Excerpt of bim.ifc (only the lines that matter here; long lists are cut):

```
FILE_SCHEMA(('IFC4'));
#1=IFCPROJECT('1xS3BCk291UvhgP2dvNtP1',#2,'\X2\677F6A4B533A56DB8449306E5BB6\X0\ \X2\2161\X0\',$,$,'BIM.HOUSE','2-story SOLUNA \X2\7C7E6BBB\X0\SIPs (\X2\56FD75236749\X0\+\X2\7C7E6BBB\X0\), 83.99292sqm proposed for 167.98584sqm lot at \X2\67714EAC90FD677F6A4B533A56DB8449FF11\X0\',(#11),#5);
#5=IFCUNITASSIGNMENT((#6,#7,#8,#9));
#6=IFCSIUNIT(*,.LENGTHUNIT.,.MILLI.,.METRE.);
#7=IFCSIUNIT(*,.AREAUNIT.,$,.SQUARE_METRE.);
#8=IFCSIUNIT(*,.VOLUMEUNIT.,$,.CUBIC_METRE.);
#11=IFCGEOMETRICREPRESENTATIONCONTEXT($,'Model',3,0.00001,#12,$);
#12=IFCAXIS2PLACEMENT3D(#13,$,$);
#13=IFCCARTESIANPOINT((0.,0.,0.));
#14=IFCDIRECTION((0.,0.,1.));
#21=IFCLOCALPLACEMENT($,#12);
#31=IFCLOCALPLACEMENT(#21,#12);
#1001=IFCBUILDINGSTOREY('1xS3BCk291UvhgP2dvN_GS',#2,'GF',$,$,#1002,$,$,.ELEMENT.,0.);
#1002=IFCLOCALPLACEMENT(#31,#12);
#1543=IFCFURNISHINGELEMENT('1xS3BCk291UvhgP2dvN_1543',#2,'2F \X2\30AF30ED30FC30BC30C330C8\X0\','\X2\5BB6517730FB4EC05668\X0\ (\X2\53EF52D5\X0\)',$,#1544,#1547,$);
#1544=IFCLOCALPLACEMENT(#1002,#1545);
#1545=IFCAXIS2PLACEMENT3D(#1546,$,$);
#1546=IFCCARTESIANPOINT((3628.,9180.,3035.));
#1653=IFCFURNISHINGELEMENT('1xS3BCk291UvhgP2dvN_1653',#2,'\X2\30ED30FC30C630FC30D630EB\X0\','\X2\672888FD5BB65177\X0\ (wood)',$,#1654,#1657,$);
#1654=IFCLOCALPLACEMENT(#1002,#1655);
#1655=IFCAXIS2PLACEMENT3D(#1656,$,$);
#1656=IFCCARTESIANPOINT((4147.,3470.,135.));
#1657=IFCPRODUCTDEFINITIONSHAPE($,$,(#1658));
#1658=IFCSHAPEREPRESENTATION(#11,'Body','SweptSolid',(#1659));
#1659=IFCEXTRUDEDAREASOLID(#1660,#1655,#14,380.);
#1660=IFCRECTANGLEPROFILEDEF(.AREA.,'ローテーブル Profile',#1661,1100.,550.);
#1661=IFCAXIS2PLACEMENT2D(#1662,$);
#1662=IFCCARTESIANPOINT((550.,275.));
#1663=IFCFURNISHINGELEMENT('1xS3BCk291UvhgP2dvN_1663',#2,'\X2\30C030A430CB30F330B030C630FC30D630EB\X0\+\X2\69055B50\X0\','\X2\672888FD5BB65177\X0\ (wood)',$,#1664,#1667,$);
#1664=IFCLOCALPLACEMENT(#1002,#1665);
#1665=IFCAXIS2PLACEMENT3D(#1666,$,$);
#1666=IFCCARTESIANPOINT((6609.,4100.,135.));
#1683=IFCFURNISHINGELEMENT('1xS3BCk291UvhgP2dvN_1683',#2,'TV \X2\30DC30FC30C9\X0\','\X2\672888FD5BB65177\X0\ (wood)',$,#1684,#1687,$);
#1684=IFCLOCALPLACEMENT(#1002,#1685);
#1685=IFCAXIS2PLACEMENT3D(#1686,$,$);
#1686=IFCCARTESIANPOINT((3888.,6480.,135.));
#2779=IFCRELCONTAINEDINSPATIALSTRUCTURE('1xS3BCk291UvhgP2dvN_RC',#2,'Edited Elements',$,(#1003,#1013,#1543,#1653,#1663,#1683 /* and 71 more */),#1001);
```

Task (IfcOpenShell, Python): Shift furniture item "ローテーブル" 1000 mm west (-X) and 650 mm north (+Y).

```python
import ifcopenshell
import ifcopenshell.api.geometry
import ifcopenshell.util.placement

model = ifcopenshell.open("bim.ifc")

item = model.by_guid("1xS3BCk291UvhgP2dvN_1653")
matrix = ifcopenshell.util.placement.get_local_placement(item.ObjectPlacement)
matrix[0, 3] -= 1000.0
matrix[1, 3] += 650.0
ifcopenshell.api.geometry.edit_object_placement(model, product=item, matrix=matrix, is_si=False)

print(ifcopenshell.util.placement.get_local_placement(item.ObjectPlacement).round(3) + 0.0)

model.write("bim_rev.ifc")
```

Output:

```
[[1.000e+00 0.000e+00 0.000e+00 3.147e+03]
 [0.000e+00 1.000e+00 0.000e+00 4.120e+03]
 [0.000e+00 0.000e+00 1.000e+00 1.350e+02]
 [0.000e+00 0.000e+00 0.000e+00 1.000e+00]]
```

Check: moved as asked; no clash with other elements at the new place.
